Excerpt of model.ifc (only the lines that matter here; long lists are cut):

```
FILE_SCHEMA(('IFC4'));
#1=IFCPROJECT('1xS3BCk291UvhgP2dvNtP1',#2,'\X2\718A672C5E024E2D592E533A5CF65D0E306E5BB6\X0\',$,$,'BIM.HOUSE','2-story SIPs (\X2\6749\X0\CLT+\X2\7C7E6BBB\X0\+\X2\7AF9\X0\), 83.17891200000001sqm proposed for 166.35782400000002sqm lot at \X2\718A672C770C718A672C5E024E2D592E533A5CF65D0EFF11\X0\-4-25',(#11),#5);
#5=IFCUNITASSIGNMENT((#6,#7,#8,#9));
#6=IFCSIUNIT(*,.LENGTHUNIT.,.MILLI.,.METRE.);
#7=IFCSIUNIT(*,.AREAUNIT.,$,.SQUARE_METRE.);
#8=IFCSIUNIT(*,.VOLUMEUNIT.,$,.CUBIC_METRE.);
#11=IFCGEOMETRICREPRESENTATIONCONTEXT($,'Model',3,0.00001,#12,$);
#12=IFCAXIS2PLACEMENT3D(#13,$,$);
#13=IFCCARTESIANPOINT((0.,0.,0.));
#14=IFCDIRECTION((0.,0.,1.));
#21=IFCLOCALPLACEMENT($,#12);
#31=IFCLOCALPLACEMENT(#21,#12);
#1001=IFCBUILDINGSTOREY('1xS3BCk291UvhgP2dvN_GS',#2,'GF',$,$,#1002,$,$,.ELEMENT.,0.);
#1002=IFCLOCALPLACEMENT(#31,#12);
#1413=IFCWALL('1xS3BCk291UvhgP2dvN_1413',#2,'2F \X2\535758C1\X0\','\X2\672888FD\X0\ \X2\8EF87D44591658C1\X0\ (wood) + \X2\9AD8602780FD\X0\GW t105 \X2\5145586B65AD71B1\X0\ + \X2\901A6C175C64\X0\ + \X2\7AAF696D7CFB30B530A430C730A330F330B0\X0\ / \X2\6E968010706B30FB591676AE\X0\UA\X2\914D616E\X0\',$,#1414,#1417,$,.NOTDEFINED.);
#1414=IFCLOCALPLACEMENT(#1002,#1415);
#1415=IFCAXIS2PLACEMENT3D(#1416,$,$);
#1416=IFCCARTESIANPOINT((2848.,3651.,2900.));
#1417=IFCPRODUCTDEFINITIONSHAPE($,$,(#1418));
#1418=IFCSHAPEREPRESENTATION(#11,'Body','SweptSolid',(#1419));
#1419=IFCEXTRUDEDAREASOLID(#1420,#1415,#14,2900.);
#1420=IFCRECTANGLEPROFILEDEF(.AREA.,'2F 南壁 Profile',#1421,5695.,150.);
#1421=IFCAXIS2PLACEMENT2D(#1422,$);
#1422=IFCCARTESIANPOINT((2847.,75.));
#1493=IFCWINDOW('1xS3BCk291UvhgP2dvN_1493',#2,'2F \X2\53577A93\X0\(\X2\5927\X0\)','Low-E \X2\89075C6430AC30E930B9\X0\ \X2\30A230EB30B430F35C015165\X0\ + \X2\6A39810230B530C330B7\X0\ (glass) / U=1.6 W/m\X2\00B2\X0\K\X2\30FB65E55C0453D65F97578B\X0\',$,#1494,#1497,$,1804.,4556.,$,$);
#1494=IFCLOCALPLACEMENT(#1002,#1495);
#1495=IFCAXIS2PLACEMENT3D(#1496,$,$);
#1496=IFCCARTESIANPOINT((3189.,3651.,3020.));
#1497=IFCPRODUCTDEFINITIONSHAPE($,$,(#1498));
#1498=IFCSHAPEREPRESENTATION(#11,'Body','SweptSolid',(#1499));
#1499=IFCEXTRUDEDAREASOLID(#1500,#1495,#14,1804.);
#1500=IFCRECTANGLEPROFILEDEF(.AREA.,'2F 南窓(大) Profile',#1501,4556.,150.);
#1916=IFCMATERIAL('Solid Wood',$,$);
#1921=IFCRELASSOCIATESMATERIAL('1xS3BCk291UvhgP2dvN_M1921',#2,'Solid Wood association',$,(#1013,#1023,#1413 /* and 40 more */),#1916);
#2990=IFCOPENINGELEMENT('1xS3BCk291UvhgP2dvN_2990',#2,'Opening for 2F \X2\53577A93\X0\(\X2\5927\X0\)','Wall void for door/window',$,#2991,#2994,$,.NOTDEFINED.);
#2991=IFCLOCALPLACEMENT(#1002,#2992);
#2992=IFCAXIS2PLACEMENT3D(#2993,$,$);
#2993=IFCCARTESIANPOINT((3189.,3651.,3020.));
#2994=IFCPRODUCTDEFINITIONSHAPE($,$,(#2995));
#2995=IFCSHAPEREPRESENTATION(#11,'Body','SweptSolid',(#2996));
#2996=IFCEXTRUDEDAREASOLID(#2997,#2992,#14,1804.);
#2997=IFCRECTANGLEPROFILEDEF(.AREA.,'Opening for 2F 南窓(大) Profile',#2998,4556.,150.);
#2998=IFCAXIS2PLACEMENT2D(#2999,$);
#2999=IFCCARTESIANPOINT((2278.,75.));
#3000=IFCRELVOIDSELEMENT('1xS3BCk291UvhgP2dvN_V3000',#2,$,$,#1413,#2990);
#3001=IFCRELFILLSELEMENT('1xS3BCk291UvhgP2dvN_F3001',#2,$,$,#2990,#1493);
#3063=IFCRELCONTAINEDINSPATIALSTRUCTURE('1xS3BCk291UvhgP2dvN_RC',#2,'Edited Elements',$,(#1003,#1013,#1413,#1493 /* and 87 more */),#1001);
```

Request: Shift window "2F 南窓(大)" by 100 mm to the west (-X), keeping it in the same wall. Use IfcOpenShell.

```python
import ifcopenshell
import ifcopenshell.api.geometry
import ifcopenshell.util.placement

model = ifcopenshell.open("model.ifc")

window = model.by_id(1493)
opening = window.FillsVoids[0].RelatingOpeningElement
wall = opening.VoidsElements[0].RelatingBuildingElement

wall_matrix = ifcopenshell.util.placement.get_local_placement(wall.ObjectPlacement)
shift = wall_matrix[:3, 0] * -100.0
before = ifcopenshell.util.placement.get_local_placement(window.ObjectPlacement)[:3, 3].copy()

# The window is not placed relative to its opening, so move both.
for product in (opening, window):
    matrix = ifcopenshell.util.placement.get_local_placement(product.ObjectPlacement)
    matrix[:3, 3] += shift
    ifcopenshell.api.geometry.edit_object_placement(model, product=product, matrix=matrix, is_si=False)

after = ifcopenshell.util.placement.get_local_placement(window.ObjectPlacement)[:3, 3]
print("window moved by", (after - before).round(3) + 0.0)

model.write("model_rev.ifc")
```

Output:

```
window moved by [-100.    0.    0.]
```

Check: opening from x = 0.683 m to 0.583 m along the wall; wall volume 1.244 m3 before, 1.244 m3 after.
